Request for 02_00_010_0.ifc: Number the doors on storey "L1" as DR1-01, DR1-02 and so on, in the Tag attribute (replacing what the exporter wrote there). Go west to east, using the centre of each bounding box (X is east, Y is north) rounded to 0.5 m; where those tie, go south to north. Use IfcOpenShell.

First a look at what the model holds.

```python
import ifcopenshell
import ifcopenshell.util.element
import ifcopenshell.util.placement

model = ifcopenshell.open("02_00_010_0.ifc")
print(model.schema)
storey = next(s for s in model.by_type("IfcBuildingStorey") if s.Name == "L1")
doors = [e for e in ifcopenshell.util.element.get_decomposition(storey) if e.is_a("IfcDoor")]
for e in sorted(doors, key=lambda e: e.id()):
    origin = ifcopenshell.util.placement.get_local_placement(e.ObjectPlacement)[:3, 3]
    print(e.id(), e.Tag, e.Name, origin.round(2) + 0.0, sep=" | ")
```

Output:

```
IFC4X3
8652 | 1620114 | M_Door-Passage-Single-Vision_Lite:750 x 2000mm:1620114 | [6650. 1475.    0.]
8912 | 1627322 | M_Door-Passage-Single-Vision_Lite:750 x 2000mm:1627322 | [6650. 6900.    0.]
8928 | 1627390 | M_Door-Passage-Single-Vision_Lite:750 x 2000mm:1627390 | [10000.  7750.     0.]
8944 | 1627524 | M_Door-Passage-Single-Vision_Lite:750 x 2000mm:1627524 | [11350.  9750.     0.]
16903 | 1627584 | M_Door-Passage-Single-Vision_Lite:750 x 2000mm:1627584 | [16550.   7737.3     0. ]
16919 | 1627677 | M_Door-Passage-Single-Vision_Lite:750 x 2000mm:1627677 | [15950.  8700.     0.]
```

```python
import ifcopenshell
import ifcopenshell.geom
import ifcopenshell.util.element
import ifcopenshell.util.shape

model = ifcopenshell.open("02_00_010_0.ifc")
settings = ifcopenshell.geom.settings()
settings.set("use-world-coords", True)


def centre(element):
    shape = ifcopenshell.geom.create_shape(settings, element)
    return ifcopenshell.util.shape.get_bbox_centroid(shape.geometry)


storey = next(s for s in model.by_type("IfcBuildingStorey") if s.Name == "L1")
doors = [e for e in ifcopenshell.util.element.get_decomposition(storey) if e.is_a("IfcDoor")]

# Insertion points can sit at a corner or the storey origin, so sort by the geometry (in metres).
centres = {e: centre(e) for e in doors}
doors.sort(key=lambda e: (round(centres[e][0] / 0.5), centres[e][1]))

for i, e in enumerate(doors, start=1):
    number = f"DR1-{i:02d}"
    e.Tag = number
    print(e.id(), number)

model.write("02_00_010_0_rev.ifc")
```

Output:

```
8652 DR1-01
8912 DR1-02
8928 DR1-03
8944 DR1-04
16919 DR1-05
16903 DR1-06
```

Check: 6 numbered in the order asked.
